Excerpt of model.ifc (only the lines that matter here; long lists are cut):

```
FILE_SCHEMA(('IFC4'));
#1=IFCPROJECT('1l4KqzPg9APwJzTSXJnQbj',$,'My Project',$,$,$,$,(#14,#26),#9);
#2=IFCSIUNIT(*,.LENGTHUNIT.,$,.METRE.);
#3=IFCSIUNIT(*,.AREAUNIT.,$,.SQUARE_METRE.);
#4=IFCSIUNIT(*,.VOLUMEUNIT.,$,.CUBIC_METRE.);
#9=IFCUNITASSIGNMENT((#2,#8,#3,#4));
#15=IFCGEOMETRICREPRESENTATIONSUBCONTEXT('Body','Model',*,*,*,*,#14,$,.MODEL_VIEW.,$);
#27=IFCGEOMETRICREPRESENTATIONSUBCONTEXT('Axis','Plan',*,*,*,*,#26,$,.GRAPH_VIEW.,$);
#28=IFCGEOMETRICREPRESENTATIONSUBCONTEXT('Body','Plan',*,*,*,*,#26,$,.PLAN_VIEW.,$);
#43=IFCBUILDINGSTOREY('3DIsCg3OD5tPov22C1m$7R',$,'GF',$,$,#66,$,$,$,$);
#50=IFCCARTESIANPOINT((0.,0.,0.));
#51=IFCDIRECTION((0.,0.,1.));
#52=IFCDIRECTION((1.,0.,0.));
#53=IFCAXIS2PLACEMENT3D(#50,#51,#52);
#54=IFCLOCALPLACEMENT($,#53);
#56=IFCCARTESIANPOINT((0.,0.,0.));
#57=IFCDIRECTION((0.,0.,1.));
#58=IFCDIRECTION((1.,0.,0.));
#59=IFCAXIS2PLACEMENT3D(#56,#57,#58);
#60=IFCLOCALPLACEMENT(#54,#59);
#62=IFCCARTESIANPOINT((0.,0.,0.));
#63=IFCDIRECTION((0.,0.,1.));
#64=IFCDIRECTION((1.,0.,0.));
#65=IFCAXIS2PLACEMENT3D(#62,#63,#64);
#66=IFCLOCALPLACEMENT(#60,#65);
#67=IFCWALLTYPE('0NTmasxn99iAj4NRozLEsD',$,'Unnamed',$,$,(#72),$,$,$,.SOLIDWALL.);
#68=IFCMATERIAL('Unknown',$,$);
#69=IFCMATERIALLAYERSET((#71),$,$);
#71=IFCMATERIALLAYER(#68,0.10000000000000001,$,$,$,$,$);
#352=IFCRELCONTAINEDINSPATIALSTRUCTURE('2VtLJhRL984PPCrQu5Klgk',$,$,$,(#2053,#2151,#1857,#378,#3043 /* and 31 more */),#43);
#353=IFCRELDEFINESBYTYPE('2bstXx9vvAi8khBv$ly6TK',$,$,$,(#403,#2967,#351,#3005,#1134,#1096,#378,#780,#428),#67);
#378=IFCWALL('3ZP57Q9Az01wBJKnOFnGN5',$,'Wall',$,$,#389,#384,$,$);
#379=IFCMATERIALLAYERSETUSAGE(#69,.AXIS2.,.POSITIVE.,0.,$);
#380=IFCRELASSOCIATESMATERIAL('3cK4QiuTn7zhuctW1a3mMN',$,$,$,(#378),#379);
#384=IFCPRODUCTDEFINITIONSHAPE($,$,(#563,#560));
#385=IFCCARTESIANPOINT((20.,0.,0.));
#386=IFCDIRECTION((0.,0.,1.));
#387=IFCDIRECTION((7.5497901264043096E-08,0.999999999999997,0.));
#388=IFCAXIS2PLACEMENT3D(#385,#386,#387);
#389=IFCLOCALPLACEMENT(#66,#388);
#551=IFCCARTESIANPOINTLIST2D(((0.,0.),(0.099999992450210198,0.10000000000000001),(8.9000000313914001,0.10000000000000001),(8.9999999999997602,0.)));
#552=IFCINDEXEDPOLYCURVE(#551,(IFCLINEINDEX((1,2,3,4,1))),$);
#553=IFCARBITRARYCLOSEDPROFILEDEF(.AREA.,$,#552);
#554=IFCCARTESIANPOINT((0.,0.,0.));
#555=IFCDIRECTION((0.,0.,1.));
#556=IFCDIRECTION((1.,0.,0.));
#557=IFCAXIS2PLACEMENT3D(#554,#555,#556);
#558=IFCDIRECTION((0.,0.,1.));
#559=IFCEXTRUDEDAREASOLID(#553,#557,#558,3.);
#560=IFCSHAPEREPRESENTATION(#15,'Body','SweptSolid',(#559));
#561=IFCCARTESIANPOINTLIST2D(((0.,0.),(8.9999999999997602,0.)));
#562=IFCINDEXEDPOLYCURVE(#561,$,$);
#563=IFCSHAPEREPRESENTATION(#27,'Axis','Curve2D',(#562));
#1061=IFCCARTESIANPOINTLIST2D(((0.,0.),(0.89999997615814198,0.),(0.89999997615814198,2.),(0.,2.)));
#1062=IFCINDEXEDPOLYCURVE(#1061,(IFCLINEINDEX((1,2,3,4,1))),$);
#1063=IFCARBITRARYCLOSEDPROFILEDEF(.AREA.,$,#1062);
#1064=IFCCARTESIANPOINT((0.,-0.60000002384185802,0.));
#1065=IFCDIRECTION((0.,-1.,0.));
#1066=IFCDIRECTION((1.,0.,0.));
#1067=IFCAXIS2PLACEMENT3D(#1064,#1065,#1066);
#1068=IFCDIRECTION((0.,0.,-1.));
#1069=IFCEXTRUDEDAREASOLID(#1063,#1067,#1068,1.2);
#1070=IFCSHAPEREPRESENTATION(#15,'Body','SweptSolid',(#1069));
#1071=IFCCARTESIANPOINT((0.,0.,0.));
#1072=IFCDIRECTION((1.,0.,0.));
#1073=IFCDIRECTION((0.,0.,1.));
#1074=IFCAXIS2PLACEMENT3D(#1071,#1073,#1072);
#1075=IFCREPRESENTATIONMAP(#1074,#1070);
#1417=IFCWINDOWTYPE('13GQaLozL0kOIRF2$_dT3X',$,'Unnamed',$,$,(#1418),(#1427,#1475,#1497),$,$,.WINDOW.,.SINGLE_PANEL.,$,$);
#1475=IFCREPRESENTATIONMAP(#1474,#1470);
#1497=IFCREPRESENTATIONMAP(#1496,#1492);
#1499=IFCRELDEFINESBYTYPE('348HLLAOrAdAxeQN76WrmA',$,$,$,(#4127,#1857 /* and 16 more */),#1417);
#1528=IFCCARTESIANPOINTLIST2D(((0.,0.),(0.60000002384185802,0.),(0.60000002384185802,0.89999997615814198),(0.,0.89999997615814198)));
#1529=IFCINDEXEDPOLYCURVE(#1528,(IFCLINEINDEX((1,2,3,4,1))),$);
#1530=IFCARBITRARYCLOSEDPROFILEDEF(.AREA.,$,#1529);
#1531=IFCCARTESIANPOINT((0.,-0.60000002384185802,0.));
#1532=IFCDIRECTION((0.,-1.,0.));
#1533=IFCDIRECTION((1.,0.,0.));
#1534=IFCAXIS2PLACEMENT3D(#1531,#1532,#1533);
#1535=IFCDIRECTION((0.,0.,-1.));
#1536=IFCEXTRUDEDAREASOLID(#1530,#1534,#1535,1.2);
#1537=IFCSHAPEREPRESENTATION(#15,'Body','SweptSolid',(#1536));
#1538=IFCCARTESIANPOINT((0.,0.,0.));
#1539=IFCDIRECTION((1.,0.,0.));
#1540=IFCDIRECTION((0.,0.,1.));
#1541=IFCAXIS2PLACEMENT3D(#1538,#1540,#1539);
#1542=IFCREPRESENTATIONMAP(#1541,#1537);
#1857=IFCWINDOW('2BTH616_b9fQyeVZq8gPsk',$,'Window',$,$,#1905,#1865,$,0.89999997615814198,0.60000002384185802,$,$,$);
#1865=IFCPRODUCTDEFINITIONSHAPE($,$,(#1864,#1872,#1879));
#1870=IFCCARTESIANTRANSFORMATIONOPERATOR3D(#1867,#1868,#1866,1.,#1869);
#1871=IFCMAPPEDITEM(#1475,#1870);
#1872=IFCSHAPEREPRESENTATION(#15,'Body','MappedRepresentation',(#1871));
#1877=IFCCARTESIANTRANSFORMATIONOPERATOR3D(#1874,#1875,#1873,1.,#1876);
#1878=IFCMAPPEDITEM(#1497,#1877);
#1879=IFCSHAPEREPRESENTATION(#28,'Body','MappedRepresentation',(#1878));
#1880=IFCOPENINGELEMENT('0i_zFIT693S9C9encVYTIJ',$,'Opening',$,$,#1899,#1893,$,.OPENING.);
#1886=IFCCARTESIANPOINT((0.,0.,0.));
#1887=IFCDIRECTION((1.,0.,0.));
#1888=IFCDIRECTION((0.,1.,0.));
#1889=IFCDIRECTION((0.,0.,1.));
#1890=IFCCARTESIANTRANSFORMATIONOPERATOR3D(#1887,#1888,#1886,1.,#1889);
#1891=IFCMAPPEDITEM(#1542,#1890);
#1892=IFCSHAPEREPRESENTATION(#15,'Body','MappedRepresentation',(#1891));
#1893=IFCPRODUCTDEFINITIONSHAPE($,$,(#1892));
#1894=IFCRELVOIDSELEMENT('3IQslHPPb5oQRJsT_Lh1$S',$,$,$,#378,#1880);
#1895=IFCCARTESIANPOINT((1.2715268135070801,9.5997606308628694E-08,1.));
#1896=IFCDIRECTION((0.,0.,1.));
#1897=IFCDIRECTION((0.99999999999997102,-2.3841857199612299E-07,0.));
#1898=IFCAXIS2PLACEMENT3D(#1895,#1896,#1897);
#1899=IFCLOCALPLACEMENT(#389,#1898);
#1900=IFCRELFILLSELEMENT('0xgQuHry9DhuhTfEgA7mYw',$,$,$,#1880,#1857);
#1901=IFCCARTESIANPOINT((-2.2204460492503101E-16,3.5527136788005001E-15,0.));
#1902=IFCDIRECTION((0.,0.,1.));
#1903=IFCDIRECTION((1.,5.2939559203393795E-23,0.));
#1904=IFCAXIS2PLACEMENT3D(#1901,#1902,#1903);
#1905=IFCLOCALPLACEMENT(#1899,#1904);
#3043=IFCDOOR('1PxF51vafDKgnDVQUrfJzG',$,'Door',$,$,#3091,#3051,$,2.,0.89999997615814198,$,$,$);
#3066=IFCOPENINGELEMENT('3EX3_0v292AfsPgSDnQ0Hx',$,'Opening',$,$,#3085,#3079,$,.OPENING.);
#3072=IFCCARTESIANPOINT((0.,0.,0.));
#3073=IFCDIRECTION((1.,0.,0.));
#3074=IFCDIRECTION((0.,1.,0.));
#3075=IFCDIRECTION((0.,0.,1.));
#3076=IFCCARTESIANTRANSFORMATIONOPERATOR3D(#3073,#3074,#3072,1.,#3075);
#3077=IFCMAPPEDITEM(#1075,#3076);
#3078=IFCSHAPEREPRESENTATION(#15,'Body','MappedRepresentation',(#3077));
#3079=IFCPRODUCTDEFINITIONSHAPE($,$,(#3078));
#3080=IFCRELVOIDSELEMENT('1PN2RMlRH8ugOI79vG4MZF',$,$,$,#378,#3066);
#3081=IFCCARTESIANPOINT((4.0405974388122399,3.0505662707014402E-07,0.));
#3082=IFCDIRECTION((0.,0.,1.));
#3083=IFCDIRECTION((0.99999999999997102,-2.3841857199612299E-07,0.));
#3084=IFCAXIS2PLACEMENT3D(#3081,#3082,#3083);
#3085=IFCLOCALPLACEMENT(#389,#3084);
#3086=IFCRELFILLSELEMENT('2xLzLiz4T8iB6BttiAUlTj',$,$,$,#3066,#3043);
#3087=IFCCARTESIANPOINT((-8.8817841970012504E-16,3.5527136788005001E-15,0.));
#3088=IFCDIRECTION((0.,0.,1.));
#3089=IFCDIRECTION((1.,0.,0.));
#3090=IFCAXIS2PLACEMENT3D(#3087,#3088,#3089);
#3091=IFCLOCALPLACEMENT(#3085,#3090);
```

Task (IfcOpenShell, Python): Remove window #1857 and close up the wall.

```python
import ifcopenshell
import ifcopenshell.api.feature
import ifcopenshell.api.root
import ifcopenshell.geom
import ifcopenshell.util.shape

model = ifcopenshell.open("model.ifc")
settings = ifcopenshell.geom.settings()


def volume(element):
    """Net volume in cubic metres, openings subtracted."""
    shape = ifcopenshell.geom.create_shape(settings, element)
    return ifcopenshell.util.shape.get_volume(shape.geometry)


window = model.by_guid("2BTH616_b9fQyeVZq8gPsk")
opening = window.FillsVoids[0].RelatingOpeningElement
wall = opening.VoidsElements[0].RelatingBuildingElement
before = volume(wall)

ifcopenshell.api.root.remove_product(model, product=window)
ifcopenshell.api.feature.remove_feature(model, feature=opening)

after = volume(wall)

print(f"wall volume {before:.3f} -> {after:.3f} m3")

model.write("model-out.ifc")
```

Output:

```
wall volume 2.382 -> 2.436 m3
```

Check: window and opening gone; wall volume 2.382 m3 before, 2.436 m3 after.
